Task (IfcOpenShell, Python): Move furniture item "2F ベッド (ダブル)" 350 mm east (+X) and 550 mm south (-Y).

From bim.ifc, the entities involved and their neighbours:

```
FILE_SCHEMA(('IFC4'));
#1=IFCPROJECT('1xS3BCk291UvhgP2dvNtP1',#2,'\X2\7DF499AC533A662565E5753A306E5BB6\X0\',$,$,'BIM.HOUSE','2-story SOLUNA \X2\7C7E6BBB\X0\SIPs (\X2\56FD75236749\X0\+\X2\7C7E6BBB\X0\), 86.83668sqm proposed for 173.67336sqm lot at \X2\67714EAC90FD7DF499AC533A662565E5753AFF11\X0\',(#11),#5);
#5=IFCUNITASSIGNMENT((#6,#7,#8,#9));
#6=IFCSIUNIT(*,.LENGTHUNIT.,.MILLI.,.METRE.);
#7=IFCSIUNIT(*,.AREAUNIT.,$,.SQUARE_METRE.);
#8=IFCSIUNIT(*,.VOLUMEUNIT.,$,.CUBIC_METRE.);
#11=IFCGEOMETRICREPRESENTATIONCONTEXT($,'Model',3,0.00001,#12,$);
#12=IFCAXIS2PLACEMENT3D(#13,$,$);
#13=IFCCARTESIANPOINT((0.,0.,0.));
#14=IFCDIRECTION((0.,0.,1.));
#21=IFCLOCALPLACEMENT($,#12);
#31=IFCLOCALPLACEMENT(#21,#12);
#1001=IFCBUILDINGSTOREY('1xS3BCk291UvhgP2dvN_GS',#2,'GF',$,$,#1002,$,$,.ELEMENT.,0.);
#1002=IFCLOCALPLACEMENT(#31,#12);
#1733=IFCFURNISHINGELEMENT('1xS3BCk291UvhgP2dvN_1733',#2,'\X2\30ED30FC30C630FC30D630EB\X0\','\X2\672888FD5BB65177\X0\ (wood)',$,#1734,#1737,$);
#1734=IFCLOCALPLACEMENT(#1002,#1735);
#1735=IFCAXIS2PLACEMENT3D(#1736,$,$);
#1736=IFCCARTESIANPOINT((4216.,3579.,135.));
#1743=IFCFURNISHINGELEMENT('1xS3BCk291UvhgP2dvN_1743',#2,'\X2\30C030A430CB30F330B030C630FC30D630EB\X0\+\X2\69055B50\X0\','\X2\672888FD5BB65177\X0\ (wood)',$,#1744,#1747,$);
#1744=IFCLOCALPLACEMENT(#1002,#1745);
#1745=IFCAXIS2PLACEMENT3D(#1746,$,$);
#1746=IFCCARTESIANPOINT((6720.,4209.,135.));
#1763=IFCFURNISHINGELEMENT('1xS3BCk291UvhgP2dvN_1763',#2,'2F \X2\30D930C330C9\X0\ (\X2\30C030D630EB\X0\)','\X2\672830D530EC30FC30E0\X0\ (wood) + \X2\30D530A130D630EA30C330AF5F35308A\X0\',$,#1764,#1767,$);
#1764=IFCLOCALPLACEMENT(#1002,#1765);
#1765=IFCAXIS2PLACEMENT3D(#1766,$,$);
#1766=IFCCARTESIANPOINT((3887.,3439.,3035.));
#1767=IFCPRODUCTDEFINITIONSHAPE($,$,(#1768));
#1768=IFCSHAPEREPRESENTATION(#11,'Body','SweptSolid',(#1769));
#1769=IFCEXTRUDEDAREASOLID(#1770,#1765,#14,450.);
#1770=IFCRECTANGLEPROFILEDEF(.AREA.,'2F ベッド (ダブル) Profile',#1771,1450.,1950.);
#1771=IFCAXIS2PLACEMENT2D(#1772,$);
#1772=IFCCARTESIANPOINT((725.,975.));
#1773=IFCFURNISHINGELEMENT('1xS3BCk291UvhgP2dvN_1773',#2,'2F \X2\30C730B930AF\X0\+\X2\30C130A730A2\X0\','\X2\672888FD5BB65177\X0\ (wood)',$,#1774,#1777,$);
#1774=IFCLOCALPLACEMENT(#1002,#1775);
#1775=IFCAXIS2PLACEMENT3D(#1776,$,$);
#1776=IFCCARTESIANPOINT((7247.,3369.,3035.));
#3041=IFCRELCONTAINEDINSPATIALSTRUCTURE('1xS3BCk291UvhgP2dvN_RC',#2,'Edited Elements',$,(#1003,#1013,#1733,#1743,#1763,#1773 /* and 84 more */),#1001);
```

```python
import ifcopenshell
import ifcopenshell.api.geometry
import ifcopenshell.util.placement
import ifcopenshell.util.unit

model = ifcopenshell.open("bim.ifc")
unit_scale = ifcopenshell.util.unit.calculate_unit_scale(model)

item = model.by_guid("1xS3BCk291UvhgP2dvN_1763")
matrix = ifcopenshell.util.placement.get_local_placement(item.ObjectPlacement)
matrix[0, 3] += 0.35 / unit_scale
matrix[1, 3] -= 0.55 / unit_scale
ifcopenshell.api.geometry.edit_object_placement(model, product=item, matrix=matrix, is_si=False)

print(ifcopenshell.util.placement.get_local_placement(item.ObjectPlacement).round(3) + 0.0)

model.write("bim_rev.ifc")
```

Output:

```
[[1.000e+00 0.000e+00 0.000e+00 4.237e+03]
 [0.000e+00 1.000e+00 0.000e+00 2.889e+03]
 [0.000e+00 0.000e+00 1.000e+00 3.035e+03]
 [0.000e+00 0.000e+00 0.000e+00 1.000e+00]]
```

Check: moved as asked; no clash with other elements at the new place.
